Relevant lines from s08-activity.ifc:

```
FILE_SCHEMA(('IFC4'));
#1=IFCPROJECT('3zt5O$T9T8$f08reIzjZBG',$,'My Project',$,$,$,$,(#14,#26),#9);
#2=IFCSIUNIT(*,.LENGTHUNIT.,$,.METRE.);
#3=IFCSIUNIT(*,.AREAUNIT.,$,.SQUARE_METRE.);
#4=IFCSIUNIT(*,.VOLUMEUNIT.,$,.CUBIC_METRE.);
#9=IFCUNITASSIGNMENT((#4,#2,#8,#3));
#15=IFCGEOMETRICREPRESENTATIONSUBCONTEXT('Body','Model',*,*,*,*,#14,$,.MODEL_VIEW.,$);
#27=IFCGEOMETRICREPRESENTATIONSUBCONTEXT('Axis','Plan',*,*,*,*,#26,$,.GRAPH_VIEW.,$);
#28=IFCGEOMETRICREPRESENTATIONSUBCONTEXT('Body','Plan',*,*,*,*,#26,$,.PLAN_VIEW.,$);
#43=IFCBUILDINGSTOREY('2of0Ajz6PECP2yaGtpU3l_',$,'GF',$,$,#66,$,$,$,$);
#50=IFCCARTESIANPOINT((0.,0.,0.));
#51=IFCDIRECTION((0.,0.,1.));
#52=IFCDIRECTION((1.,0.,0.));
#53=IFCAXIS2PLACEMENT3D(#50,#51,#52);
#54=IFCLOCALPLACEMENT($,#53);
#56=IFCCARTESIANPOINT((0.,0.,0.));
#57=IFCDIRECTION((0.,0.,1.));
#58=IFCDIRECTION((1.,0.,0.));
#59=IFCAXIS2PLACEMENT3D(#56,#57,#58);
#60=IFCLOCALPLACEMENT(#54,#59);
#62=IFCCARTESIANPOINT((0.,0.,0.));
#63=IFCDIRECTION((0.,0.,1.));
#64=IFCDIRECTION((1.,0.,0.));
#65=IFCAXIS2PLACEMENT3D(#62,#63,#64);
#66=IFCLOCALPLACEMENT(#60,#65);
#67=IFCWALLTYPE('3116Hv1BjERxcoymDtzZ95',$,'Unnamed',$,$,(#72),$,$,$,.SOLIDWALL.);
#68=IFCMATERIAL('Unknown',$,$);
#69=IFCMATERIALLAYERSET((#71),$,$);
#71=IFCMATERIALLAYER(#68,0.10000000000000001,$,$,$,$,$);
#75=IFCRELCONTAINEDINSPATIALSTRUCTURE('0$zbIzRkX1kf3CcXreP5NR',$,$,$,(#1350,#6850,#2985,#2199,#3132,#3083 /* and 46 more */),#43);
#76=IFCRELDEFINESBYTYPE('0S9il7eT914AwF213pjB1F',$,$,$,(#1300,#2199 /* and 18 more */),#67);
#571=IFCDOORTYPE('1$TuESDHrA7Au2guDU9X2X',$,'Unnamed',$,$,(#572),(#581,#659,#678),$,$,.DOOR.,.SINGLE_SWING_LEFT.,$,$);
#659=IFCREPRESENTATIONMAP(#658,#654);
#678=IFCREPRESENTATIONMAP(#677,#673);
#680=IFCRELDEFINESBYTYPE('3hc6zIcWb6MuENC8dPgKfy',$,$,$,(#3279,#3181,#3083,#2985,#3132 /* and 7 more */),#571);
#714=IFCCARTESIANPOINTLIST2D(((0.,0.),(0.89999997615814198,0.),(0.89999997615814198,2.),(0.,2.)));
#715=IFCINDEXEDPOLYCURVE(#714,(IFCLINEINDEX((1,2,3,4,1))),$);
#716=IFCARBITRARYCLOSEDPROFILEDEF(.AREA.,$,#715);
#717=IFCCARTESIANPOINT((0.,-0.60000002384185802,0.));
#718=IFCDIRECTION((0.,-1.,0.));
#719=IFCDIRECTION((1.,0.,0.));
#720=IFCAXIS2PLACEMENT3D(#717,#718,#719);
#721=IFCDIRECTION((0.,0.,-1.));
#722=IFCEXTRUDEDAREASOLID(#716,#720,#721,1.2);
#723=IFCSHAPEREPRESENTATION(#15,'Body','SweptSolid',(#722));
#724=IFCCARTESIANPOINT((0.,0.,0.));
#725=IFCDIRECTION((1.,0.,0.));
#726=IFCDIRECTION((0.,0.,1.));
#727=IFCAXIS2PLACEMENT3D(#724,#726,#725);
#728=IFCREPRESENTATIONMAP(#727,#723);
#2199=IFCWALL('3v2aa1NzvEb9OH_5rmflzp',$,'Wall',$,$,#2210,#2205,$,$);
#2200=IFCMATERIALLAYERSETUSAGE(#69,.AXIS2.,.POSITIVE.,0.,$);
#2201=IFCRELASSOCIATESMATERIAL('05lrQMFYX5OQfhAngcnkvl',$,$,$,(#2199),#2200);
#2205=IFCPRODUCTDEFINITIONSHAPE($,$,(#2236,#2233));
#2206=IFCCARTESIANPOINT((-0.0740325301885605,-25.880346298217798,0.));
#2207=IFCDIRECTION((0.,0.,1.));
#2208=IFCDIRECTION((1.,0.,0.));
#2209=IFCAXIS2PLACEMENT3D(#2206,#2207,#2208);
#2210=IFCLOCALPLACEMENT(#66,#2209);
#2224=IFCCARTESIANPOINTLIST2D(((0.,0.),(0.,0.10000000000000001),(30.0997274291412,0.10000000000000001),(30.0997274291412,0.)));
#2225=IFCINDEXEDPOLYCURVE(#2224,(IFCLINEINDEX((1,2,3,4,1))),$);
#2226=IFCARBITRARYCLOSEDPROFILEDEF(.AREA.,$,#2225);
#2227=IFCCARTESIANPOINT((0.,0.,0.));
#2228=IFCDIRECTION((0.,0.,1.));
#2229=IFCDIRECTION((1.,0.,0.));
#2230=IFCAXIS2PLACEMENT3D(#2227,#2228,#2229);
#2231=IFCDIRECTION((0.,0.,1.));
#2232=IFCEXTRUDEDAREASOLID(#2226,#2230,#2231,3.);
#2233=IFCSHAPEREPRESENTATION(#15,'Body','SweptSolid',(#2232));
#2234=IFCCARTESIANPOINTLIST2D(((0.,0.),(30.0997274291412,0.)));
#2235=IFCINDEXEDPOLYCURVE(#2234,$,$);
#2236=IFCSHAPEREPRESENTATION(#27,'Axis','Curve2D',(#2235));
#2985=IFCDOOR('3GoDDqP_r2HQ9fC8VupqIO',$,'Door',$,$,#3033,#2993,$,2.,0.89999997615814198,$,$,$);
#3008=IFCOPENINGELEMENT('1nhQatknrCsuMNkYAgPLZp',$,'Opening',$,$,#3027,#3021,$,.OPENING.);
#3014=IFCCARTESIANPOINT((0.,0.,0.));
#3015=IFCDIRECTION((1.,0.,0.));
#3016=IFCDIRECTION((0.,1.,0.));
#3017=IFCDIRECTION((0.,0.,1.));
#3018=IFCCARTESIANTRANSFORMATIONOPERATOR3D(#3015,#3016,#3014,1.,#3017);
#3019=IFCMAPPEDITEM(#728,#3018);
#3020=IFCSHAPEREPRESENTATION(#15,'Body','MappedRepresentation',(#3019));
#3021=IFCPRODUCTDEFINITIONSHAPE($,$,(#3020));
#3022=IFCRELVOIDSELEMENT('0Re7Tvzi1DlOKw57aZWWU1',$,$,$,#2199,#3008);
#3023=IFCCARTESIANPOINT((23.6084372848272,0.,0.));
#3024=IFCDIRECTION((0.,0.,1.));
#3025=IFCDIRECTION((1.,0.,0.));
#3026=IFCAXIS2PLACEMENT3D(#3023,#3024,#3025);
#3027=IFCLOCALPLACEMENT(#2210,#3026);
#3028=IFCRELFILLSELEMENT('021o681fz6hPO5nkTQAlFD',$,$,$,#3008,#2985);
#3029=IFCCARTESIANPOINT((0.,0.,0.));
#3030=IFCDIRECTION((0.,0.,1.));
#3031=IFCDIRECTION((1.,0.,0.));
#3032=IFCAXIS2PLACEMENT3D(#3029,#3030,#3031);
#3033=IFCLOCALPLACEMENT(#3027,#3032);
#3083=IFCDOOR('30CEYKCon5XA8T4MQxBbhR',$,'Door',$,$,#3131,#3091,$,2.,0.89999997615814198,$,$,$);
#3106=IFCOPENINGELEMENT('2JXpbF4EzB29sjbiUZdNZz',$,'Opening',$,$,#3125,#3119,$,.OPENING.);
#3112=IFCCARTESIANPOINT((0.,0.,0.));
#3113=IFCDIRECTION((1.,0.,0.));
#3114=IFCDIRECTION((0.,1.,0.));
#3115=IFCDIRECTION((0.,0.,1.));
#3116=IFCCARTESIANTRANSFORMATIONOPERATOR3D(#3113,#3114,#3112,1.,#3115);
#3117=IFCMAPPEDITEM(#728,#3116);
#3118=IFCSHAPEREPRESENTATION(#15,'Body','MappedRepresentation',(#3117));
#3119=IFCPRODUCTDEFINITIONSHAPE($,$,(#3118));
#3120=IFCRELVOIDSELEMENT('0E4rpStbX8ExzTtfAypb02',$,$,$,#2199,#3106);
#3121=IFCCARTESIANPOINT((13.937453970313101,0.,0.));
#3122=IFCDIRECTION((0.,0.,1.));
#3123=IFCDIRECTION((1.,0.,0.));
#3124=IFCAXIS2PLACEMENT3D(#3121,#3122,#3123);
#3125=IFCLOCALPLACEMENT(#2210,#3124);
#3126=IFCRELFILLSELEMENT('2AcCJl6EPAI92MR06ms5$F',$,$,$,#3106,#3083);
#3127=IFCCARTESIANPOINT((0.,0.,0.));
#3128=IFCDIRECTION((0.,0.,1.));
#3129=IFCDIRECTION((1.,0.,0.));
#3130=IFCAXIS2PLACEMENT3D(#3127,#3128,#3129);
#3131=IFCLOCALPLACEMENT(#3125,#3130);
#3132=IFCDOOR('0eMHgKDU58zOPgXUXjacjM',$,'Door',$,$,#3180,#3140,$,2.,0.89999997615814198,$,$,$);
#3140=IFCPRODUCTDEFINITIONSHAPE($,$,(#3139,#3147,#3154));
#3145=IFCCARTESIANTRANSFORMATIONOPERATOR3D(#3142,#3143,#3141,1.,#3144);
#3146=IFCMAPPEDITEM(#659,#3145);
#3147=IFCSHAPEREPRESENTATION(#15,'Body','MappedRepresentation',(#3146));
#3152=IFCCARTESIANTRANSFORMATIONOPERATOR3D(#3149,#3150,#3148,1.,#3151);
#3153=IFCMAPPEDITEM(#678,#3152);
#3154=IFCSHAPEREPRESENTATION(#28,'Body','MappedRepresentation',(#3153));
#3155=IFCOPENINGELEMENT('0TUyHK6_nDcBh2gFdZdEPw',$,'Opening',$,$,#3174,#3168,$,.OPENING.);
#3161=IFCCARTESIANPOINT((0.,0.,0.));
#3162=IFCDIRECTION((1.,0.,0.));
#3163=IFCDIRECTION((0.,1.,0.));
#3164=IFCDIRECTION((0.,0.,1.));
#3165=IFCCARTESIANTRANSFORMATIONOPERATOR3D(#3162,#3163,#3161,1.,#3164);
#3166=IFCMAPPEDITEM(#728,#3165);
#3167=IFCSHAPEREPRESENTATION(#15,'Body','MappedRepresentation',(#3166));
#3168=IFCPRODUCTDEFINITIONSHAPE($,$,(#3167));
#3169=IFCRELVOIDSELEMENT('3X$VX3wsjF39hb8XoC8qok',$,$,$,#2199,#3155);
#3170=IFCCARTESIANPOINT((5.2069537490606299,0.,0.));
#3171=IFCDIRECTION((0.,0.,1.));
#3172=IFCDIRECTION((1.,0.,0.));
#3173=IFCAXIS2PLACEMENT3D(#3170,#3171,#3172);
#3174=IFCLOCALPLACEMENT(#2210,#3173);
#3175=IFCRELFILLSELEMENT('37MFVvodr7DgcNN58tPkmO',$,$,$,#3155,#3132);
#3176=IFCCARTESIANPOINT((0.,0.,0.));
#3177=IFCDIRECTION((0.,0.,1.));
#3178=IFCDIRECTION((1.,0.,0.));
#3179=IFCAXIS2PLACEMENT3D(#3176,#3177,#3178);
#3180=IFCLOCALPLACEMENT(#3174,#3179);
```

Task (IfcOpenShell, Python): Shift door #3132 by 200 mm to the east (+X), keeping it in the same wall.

```python
import ifcopenshell
import ifcopenshell.api.geometry
import ifcopenshell.util.placement

model = ifcopenshell.open("s08-activity.ifc")

door = model.by_id(3132)
opening = door.FillsVoids[0].RelatingOpeningElement
wall = opening.VoidsElements[0].RelatingBuildingElement

wall_matrix = ifcopenshell.util.placement.get_local_placement(wall.ObjectPlacement)
shift = wall_matrix[:3, 0] * 0.2
before = ifcopenshell.util.placement.get_local_placement(door.ObjectPlacement)[:3, 3].copy()

# The door is placed relative to its opening, so it follows when the opening moves.
matrix = ifcopenshell.util.placement.get_local_placement(opening.ObjectPlacement)
matrix[:3, 3] += shift
ifcopenshell.api.geometry.edit_object_placement(
    model, product=opening, matrix=matrix, is_si=False, should_transform_children=True
)

after = ifcopenshell.util.placement.get_local_placement(door.ObjectPlacement)[:3, 3]
print("door moved by", (after - before).round(3) + 0.0)

model.write("s08-activity_edited.ifc")
```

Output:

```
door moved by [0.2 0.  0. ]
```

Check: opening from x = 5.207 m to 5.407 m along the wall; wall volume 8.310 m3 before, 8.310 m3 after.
